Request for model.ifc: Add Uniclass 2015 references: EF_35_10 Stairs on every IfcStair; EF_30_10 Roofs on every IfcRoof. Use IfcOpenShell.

First a look at what the model holds.

```python
import ifcopenshell

model = ifcopenshell.open("model.ifc")
print(model.schema)
print("classifications:", [c.Name for c in model.by_type("IfcClassification")])
for ifc_class in ("IfcDoor", "IfcRoof", "IfcStair", "IfcWall", "IfcWindow"):
    print(ifc_class, len(model.by_type(ifc_class)))
```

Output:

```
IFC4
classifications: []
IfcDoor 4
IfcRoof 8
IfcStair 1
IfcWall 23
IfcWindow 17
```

```python
import ifcopenshell
import ifcopenshell.api.classification

model = ifcopenshell.open("model.ifc")

system = ifcopenshell.api.classification.add_classification(model, classification="Uniclass 2015")

codes = {
    "IfcStair": ("EF_35_10", "Stairs"),
    "IfcRoof": ("EF_30_10", "Roofs"),
}
for ifc_class, (code, name) in codes.items():
    products = model.by_type(ifc_class)
    ifcopenshell.api.classification.add_reference(
        model, products=products, classification=system, identification=code, name=name
    )
    print(code, len(products))

model.write("model-out.ifc")
```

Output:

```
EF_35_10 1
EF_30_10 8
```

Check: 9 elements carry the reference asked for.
